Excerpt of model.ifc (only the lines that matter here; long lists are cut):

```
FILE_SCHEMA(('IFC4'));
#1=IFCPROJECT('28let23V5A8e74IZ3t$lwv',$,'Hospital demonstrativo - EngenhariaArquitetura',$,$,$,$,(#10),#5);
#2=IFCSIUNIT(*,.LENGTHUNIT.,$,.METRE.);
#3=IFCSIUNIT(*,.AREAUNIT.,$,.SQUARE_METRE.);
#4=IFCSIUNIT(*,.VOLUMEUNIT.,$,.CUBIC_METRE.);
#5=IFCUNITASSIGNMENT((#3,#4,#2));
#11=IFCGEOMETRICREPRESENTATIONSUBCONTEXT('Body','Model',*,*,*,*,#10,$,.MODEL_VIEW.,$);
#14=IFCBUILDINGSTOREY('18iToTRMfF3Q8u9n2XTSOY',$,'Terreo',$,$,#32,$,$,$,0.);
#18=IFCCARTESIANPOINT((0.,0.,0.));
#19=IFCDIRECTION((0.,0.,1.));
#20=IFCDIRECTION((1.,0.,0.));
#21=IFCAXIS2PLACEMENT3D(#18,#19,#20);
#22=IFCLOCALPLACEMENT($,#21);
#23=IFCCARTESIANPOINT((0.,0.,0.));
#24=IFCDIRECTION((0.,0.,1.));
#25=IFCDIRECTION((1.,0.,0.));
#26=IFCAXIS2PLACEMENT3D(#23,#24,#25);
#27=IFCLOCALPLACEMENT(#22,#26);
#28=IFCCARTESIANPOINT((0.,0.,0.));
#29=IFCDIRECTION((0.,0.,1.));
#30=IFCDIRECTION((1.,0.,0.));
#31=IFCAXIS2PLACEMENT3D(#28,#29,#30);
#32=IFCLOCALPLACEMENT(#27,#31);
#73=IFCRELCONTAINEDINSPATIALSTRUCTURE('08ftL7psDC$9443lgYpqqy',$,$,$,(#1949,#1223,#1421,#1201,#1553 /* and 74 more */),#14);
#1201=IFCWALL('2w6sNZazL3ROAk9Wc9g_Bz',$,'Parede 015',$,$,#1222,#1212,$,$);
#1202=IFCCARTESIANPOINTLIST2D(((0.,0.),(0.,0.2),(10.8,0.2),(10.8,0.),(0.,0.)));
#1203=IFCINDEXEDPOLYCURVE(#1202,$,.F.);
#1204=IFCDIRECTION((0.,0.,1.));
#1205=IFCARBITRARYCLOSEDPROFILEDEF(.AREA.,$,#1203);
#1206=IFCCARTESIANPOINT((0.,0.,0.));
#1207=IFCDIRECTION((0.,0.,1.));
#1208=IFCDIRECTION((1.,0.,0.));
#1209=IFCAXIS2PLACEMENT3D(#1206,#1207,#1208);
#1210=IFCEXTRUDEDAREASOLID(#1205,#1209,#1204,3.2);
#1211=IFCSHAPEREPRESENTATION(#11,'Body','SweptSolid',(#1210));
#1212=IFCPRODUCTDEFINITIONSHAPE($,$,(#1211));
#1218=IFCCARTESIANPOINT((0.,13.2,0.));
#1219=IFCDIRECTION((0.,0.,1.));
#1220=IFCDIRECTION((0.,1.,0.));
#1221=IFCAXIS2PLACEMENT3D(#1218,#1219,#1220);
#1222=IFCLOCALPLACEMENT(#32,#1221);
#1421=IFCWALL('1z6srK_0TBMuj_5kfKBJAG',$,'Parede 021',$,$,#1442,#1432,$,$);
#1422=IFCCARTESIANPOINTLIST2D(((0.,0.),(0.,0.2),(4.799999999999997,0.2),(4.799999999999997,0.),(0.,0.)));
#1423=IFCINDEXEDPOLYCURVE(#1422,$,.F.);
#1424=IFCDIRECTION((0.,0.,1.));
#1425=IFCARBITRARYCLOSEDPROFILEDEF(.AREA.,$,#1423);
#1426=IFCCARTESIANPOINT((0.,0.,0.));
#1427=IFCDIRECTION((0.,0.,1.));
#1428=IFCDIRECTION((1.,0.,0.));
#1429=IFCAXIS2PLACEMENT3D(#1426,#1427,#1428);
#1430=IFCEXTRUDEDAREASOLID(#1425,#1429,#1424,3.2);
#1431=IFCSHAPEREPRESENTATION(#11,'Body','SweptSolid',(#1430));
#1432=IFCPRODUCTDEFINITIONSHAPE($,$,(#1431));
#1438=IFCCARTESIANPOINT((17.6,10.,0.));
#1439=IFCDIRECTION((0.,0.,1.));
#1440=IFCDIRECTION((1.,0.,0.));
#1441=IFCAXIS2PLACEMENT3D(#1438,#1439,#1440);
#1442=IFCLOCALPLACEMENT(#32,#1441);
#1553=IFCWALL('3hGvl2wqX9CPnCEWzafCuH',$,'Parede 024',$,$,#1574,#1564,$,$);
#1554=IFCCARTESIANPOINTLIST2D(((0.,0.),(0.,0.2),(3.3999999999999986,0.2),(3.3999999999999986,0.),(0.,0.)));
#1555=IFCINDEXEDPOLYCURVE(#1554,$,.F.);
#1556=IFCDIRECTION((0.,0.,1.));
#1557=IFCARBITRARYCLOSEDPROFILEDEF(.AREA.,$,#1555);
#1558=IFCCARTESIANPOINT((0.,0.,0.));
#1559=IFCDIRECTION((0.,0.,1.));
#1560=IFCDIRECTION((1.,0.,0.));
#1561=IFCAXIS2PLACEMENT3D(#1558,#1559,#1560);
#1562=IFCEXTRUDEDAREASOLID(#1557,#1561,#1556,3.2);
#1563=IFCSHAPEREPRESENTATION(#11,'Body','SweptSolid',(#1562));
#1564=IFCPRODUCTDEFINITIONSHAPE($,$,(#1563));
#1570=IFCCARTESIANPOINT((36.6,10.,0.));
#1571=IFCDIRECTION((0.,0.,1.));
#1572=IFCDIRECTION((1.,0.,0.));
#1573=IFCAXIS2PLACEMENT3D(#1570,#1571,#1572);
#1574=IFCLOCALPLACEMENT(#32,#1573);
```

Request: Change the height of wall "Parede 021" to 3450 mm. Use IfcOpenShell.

```python
import ifcopenshell
import ifcopenshell.geom
import ifcopenshell.util.representation
import ifcopenshell.util.shape

model = ifcopenshell.open("model.ifc")
settings = ifcopenshell.geom.settings()


def volume(element):
    """Net volume in cubic metres, openings subtracted."""
    shape = ifcopenshell.geom.create_shape(settings, element)
    return ifcopenshell.util.shape.get_volume(shape.geometry)


wall = model.by_id(1421)
before = volume(wall)

body = ifcopenshell.util.representation.get_representation(wall, "Model", "Body")
solid = body.Items[0]
old_height = solid.Depth
solid.Depth = 3.45
after = volume(wall)

print(f"height {old_height:g} -> {solid.Depth:g}, volume {before:.3f} -> {after:.3f} m3")

model.write("model-out.ifc")
```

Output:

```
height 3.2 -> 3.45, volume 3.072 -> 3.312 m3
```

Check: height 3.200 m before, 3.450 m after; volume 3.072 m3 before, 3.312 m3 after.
